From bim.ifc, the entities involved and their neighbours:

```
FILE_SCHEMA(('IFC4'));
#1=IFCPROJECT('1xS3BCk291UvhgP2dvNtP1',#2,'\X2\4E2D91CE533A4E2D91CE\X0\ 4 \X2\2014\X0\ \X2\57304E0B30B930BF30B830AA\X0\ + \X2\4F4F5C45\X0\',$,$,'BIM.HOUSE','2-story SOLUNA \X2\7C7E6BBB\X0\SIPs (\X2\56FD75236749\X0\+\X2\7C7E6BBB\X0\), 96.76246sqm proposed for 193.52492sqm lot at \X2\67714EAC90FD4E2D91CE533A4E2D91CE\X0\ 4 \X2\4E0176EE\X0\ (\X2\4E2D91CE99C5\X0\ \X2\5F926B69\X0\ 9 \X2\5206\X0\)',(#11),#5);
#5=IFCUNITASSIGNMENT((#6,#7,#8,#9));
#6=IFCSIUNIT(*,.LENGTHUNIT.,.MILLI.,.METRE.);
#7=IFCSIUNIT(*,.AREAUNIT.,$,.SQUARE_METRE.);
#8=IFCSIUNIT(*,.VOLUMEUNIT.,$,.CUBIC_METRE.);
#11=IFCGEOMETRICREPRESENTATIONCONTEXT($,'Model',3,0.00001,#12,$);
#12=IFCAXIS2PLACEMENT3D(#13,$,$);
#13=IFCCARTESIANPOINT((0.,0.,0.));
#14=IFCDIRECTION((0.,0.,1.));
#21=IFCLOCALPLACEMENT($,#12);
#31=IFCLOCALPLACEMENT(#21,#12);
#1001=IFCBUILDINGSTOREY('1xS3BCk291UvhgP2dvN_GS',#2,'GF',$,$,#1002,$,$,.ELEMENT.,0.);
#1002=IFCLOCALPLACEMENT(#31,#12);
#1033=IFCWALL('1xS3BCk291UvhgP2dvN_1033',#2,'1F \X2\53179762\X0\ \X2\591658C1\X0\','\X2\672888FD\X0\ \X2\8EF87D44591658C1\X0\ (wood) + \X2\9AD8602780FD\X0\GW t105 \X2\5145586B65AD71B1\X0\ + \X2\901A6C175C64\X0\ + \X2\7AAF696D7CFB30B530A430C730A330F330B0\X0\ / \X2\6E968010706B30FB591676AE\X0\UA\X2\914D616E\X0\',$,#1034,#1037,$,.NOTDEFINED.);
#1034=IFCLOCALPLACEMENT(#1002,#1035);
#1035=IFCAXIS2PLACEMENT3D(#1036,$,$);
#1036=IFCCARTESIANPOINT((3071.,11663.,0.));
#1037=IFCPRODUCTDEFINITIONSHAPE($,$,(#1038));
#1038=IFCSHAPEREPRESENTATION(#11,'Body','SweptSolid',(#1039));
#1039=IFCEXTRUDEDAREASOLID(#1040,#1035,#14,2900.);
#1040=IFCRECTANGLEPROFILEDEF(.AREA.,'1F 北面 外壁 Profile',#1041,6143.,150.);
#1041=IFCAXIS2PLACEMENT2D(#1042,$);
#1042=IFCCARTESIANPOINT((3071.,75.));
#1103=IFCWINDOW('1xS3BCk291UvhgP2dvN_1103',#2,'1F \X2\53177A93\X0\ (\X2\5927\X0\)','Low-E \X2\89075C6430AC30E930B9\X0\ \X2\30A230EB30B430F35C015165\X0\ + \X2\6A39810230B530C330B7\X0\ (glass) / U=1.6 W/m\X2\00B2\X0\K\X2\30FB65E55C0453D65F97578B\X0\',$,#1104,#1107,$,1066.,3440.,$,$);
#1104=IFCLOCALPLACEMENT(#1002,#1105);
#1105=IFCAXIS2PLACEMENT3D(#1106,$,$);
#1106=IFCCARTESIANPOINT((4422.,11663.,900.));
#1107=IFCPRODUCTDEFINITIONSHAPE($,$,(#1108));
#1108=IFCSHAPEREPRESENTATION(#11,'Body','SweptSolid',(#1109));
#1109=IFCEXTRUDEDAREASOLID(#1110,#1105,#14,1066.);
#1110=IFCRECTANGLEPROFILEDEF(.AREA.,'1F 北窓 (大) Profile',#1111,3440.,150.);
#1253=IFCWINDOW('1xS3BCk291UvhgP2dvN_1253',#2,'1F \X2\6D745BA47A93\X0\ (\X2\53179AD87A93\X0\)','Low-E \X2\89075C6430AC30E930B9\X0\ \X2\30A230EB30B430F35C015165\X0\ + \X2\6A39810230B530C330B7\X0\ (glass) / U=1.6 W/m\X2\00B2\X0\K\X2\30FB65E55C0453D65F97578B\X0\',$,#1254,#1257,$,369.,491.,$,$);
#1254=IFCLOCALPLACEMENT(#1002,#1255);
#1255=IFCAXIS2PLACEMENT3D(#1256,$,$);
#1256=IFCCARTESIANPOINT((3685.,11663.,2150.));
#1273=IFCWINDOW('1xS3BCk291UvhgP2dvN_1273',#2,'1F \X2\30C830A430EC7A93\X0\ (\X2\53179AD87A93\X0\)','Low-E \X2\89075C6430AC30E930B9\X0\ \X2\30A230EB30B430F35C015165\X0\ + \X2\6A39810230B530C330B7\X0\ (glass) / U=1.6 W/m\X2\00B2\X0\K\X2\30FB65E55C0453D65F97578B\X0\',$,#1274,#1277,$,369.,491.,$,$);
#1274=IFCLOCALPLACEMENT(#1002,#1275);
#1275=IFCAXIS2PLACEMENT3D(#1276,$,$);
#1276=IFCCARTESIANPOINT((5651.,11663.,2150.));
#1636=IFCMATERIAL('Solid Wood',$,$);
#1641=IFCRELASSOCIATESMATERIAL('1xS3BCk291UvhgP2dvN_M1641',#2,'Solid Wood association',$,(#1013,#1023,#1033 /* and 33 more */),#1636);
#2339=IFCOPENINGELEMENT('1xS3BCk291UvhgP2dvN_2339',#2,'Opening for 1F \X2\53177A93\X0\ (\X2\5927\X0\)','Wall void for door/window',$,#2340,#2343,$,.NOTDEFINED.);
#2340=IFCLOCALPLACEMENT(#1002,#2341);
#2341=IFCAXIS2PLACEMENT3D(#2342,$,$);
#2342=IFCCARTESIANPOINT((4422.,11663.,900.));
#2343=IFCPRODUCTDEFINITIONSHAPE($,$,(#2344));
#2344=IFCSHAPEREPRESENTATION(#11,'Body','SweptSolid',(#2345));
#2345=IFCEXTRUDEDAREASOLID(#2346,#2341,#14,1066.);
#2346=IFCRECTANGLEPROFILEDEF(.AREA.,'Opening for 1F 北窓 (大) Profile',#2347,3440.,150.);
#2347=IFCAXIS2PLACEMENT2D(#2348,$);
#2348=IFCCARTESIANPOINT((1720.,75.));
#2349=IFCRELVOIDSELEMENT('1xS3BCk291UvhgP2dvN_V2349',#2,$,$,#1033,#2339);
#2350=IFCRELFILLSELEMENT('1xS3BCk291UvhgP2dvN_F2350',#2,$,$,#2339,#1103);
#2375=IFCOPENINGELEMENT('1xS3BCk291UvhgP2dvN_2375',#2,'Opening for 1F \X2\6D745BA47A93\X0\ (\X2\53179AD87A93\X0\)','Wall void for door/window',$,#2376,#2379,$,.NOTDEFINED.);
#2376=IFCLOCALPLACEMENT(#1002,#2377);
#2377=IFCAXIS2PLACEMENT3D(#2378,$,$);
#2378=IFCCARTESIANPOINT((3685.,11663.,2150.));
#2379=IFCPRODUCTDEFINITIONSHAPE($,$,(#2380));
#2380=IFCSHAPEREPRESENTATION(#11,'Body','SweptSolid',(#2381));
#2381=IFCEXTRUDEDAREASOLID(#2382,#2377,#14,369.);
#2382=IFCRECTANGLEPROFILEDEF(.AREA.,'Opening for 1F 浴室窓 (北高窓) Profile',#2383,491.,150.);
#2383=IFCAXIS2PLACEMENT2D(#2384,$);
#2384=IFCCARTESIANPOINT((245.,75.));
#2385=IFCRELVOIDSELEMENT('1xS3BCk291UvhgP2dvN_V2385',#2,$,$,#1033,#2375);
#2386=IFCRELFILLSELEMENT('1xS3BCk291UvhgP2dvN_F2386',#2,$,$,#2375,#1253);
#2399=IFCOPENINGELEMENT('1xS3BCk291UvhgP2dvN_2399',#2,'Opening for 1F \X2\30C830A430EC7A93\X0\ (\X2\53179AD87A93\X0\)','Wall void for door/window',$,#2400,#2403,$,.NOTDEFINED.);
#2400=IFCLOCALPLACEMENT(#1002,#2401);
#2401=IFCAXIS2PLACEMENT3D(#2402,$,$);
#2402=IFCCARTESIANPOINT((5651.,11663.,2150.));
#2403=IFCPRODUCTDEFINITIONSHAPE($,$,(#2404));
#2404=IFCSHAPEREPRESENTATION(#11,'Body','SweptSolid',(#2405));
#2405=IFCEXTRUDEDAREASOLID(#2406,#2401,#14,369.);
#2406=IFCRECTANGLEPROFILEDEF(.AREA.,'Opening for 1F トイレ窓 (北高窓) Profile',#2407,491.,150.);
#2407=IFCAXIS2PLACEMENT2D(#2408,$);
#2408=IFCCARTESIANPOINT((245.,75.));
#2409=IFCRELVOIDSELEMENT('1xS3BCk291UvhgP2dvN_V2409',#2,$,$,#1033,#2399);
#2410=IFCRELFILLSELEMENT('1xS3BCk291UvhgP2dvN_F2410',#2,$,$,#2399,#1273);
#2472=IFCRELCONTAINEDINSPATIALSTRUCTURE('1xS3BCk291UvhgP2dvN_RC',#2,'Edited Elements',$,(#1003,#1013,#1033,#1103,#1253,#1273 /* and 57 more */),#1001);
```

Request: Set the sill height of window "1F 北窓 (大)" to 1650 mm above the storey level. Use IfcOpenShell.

```python
import numpy as np
import ifcopenshell
import ifcopenshell.api.geometry
import ifcopenshell.geom
import ifcopenshell.util.element
import ifcopenshell.util.placement
import ifcopenshell.util.shape
import ifcopenshell.util.unit

model = ifcopenshell.open("bim.ifc")
unit_scale = ifcopenshell.util.unit.calculate_unit_scale(model)

window = model.by_id(1103)
opening = window.FillsVoids[0].RelatingOpeningElement
storey = ifcopenshell.util.element.get_container(window, ifc_class="IfcBuildingStorey")
level = ifcopenshell.util.placement.get_local_placement(storey.ObjectPlacement)[2, 3]

# The opening's origin need not be at the sill, so measure its lowest point.
shape = ifcopenshell.geom.create_shape(ifcopenshell.geom.settings(), opening)
bottom = ifcopenshell.util.shape.get_shape_bottom_elevation(shape, shape.geometry) / unit_scale
dz = level + 1.65 / unit_scale - bottom

shift = np.array([0.0, 0.0, dz])
# The window is not placed relative to its opening, so move both.
for product in (opening, window):
    matrix = ifcopenshell.util.placement.get_local_placement(product.ObjectPlacement)
    matrix[:3, 3] += shift
    ifcopenshell.api.geometry.edit_object_placement(model, product=product, matrix=matrix, is_si=False)

print(f"moved by {dz * unit_scale:+.3f} m")

model.write("bim_edited.ifc")
```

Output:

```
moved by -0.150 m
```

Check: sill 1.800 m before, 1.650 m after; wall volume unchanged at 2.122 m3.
